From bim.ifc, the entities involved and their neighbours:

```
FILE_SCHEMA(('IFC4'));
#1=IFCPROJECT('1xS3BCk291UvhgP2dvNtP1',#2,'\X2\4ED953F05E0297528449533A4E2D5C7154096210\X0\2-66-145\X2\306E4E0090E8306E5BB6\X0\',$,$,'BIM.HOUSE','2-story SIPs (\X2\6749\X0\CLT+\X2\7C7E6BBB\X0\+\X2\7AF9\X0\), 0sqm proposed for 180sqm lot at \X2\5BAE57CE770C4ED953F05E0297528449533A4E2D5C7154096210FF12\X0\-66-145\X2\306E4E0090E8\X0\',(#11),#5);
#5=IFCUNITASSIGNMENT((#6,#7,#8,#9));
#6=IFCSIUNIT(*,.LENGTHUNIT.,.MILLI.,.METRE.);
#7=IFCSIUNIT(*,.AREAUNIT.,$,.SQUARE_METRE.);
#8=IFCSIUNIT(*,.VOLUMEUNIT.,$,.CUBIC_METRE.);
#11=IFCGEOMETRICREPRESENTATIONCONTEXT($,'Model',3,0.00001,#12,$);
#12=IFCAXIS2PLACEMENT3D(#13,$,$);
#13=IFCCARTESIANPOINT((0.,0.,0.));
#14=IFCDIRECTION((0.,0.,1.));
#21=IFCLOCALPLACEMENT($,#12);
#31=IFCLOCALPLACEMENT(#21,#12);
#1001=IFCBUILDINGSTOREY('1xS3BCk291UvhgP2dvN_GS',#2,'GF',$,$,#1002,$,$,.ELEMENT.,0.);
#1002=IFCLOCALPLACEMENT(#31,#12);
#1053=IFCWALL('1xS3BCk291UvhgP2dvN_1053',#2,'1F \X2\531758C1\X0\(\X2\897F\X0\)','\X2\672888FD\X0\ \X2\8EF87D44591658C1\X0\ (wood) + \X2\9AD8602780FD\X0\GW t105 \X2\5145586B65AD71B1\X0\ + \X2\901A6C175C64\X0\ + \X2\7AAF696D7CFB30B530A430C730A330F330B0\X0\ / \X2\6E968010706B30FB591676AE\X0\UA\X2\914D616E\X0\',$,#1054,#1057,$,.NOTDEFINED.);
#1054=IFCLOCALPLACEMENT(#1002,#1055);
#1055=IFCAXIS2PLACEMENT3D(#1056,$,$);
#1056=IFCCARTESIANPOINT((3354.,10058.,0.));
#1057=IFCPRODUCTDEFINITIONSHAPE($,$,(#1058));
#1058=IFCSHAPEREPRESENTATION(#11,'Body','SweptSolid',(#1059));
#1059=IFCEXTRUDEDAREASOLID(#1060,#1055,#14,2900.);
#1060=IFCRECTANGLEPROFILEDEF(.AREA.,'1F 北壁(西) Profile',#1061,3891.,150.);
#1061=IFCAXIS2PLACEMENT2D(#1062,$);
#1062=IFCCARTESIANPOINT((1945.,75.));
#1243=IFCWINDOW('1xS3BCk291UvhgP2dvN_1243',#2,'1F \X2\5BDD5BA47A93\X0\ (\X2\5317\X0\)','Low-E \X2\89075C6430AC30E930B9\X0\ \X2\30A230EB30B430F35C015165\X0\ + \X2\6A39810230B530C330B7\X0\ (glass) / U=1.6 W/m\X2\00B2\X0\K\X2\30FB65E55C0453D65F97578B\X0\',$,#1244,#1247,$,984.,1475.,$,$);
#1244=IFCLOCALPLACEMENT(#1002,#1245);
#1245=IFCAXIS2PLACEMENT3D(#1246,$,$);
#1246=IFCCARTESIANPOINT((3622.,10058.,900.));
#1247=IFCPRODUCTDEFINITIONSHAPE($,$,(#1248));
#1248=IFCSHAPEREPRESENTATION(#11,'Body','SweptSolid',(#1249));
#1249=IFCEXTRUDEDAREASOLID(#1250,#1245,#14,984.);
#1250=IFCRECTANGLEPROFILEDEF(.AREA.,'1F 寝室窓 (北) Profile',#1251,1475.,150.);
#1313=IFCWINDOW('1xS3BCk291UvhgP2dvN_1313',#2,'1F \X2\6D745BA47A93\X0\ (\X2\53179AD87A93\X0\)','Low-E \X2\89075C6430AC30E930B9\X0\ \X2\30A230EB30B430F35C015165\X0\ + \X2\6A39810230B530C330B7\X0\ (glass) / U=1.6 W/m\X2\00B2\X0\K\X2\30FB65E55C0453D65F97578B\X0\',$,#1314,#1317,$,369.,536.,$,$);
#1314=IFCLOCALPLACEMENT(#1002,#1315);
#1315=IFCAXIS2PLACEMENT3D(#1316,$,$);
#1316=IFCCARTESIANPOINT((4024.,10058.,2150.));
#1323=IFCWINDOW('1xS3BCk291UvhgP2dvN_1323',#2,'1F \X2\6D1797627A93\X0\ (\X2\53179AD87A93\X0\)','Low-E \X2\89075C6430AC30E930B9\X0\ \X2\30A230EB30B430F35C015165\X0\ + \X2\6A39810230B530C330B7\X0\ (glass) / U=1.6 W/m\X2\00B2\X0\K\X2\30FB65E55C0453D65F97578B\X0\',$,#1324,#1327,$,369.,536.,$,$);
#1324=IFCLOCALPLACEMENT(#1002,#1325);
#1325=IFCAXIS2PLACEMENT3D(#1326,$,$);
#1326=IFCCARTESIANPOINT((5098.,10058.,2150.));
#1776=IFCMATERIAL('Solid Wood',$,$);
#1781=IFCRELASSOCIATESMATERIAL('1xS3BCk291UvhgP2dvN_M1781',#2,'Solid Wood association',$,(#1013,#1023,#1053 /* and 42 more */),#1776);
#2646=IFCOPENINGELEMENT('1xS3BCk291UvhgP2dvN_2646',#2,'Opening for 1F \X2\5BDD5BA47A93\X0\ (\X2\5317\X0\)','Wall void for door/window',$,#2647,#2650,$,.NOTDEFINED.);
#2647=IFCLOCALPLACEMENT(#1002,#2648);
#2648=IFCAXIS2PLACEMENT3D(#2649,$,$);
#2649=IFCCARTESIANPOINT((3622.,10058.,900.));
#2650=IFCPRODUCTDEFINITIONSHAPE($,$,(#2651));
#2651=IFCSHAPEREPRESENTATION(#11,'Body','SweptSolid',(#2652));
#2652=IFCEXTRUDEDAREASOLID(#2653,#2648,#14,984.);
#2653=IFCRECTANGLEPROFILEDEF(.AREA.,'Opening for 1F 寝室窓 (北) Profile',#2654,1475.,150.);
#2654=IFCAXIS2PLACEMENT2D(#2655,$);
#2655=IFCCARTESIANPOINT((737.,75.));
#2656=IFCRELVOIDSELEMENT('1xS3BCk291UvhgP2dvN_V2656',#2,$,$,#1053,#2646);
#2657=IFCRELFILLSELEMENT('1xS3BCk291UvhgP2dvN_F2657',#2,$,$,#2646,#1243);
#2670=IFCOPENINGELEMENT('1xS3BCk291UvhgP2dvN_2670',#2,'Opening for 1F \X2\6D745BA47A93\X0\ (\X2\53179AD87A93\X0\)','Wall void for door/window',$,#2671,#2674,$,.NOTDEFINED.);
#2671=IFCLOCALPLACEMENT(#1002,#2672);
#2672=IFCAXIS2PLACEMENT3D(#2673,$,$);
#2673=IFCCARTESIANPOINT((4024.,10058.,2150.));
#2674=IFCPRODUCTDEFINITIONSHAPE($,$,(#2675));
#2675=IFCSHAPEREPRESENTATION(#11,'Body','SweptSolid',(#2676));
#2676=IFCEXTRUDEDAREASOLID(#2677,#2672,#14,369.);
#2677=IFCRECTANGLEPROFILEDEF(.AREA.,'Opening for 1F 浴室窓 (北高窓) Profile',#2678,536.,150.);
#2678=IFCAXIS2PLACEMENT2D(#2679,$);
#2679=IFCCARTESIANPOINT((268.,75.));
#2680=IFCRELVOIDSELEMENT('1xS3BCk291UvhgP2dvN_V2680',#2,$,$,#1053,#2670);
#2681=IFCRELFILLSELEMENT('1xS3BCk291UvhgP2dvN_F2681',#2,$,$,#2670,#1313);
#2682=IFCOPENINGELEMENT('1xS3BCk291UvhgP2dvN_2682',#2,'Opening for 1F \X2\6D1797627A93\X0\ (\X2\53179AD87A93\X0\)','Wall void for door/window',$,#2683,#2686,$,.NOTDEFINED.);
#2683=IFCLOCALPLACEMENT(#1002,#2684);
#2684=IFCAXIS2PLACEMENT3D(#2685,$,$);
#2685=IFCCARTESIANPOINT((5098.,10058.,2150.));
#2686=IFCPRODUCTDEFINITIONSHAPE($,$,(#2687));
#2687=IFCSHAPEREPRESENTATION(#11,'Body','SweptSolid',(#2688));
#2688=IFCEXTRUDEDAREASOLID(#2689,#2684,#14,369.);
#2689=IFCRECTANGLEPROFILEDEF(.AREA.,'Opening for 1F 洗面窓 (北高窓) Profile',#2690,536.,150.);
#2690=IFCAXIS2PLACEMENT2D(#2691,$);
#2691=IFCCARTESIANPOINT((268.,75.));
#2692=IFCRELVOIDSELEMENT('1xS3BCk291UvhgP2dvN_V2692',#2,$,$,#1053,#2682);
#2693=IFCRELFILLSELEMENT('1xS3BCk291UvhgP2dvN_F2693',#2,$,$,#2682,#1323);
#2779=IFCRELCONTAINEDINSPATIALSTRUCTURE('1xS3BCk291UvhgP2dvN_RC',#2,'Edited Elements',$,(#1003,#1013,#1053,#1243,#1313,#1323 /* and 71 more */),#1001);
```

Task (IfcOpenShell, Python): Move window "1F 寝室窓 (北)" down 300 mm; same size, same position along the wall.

```python
import numpy as np
import ifcopenshell
import ifcopenshell.api.geometry
import ifcopenshell.util.placement
import ifcopenshell.util.unit

model = ifcopenshell.open("bim.ifc")
unit_scale = ifcopenshell.util.unit.calculate_unit_scale(model)

window = model.by_guid("1xS3BCk291UvhgP2dvN_1243")
opening = window.FillsVoids[0].RelatingOpeningElement
dz = -0.3 / unit_scale

shift = np.array([0.0, 0.0, dz])
# The window is not placed relative to its opening, so move both.
for product in (opening, window):
    matrix = ifcopenshell.util.placement.get_local_placement(product.ObjectPlacement)
    matrix[:3, 3] += shift
    ifcopenshell.api.geometry.edit_object_placement(model, product=product, matrix=matrix, is_si=False)

print(f"moved by {dz * unit_scale:+.3f} m")

model.write("bim_rev.ifc")
```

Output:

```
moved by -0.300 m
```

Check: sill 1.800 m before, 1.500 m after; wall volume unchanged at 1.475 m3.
